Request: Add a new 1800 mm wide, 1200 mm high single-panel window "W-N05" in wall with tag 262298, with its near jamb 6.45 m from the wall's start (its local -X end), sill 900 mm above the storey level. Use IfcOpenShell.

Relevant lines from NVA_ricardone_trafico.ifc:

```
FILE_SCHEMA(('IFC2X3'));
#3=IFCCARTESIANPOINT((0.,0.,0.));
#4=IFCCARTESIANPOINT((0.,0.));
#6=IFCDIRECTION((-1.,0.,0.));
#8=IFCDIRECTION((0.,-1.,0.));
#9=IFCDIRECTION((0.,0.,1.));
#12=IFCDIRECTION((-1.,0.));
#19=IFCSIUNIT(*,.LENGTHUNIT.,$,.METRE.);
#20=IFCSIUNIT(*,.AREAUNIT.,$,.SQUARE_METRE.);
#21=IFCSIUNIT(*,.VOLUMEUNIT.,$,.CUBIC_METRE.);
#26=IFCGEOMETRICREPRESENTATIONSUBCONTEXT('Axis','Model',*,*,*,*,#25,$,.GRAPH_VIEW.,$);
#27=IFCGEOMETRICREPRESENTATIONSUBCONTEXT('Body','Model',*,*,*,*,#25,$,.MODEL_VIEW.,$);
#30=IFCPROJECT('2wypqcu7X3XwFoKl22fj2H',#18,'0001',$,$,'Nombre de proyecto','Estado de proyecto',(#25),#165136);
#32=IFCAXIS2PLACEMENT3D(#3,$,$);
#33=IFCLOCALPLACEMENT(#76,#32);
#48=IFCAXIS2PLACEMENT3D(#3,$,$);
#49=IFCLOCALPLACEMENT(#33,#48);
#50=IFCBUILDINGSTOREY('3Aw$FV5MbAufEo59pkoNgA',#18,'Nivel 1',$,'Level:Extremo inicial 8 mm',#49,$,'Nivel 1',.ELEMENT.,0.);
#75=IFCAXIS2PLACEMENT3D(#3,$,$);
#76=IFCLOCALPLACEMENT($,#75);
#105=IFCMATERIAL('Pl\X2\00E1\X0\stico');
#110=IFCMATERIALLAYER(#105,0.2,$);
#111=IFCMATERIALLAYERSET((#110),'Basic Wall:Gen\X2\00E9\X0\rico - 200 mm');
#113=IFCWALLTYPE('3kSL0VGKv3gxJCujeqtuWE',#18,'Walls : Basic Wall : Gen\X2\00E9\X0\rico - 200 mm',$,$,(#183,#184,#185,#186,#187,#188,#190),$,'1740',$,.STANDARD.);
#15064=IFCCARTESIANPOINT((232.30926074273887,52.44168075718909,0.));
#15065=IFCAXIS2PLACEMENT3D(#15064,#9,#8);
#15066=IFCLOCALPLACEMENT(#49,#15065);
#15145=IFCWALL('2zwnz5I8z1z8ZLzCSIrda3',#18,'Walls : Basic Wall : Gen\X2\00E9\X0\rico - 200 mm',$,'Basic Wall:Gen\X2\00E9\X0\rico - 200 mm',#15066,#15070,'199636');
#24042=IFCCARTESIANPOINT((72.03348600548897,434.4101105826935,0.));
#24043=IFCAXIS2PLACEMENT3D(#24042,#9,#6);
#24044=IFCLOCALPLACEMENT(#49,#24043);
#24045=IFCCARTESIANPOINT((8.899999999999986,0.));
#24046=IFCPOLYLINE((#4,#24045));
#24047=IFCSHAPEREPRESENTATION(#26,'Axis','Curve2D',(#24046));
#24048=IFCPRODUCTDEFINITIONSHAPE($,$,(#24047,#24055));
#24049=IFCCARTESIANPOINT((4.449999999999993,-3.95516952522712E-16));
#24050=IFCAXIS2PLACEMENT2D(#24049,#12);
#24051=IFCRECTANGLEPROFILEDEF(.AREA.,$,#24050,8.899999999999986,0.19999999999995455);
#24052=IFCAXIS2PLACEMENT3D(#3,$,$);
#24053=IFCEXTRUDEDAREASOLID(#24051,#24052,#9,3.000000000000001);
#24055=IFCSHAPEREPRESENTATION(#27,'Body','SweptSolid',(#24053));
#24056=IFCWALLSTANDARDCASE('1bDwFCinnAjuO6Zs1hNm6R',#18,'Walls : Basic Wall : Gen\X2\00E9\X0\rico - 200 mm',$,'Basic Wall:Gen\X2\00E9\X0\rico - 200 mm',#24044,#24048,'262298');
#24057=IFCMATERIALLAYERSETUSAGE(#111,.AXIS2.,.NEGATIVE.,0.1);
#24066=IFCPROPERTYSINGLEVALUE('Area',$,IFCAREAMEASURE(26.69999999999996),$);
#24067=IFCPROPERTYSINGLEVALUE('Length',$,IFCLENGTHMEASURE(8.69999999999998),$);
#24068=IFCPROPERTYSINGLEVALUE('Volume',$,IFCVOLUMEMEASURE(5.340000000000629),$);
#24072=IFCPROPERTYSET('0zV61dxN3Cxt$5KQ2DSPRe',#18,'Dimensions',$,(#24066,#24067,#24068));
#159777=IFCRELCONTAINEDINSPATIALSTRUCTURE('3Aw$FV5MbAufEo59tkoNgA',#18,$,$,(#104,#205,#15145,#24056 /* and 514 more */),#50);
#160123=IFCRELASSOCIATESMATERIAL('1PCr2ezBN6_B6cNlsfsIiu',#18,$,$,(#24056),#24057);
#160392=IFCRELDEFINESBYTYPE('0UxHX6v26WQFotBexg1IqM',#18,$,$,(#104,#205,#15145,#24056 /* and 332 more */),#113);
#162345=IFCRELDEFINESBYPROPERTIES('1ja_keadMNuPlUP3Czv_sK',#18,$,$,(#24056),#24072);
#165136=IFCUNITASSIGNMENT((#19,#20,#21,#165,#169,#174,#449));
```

```python
import numpy as np
import ifcopenshell
import ifcopenshell.api.feature
import ifcopenshell.api.geometry
import ifcopenshell.api.pset
import ifcopenshell.api.root
import ifcopenshell.api.spatial
import ifcopenshell.api.type
import ifcopenshell.geom
import ifcopenshell.util.element
import ifcopenshell.util.placement
import ifcopenshell.util.representation
import ifcopenshell.util.shape
import ifcopenshell.util.unit

model = ifcopenshell.open("NVA_ricardone_trafico.ifc")
unit_scale = ifcopenshell.util.unit.calculate_unit_scale(model)
area_scale = ifcopenshell.util.unit.calculate_unit_scale(model, "AREAUNIT")
volume_scale = ifcopenshell.util.unit.calculate_unit_scale(model, "VOLUMEUNIT")
settings = ifcopenshell.geom.settings()


def volume(element):
    """Net volume in cubic metres, openings subtracted."""
    shape = ifcopenshell.geom.create_shape(settings, element)
    return ifcopenshell.util.shape.get_volume(shape.geometry)


wall = model.by_guid("1bDwFCinnAjuO6Zs1hNm6R")
storey = ifcopenshell.util.element.get_container(wall, ifc_class="IfcBuildingStorey")
context = ifcopenshell.util.representation.get_context(model, "Model", "Body", "MODEL_VIEW")
before = volume(wall)

width, height, from_end, sill = 1.8, 1.2, 6.45, 0.9  # metres

# The wall runs along its own X axis, and the end named is its -X end.
wall_shape = ifcopenshell.geom.create_shape(settings, wall)
x, y, z = ifcopenshell.util.shape.get_vertices(wall_shape.geometry).T
start = x.min() + from_end
face, thickness = float(y.min()), float(y.max() - y.min())
wall_matrix = ifcopenshell.util.placement.get_local_placement(wall.ObjectPlacement)
level = ifcopenshell.util.placement.get_local_placement(storey.ObjectPlacement)[2, 3]


def in_wall(x, y):
    """Placement at x, y metres in the wall's axes, at sill height."""
    matrix = wall_matrix.copy()
    matrix[:, 3] = wall_matrix @ np.array([x / unit_scale, y / unit_scale, 0.0, 1.0])
    matrix[2, 3] = level + sill / unit_scale
    return matrix


# Opening: a box that overshoots both wall faces by 50 mm.
opening = ifcopenshell.api.root.create_entity(model, ifc_class="IfcOpeningElement")
box = ifcopenshell.api.geometry.add_wall_representation(
    model, context=context, length=width, height=height, thickness=thickness + 0.1
)
ifcopenshell.api.geometry.assign_representation(model, product=opening, representation=box)
ifcopenshell.api.geometry.edit_object_placement(model, product=opening, matrix=in_wall(start, face - 0.05), is_si=False)
ifcopenshell.api.feature.add_feature(model, feature=opening, element=wall)

window = ifcopenshell.api.root.create_entity(model, ifc_class="IfcWindow", name="W-N05")
window.OverallWidth, window.OverallHeight = width / unit_scale, height / unit_scale
body = ifcopenshell.api.geometry.add_window_representation(
    model,
    context=context,
    overall_width=window.OverallWidth,
    overall_height=window.OverallHeight,
    partition_type="SINGLE_PANEL",
)
ifcopenshell.api.geometry.assign_representation(model, product=window, representation=body)
ifcopenshell.api.spatial.assign_container(model, products=[window], relating_structure=storey)
fills = ifcopenshell.api.feature.add_filling(model, opening=opening, element=window)
fills.OwnerHistory = window.OwnerHistory  # required in IFC2X3

# IFC2X3 keeps the operation on the window style.
style = ifcopenshell.api.root.create_entity(model, ifc_class="IfcWindowStyle", name="W-N05")
style.OperationType, style.ConstructionType = "SINGLE_PANEL", "NOTDEFINED"
style.ParameterTakesPrecedence = style.Sizeable = False
ifcopenshell.api.type.assign_type(model, related_objects=[window], relating_type=style)

# Centre the window in the wall's thickness.
ifcopenshell.api.geometry.edit_object_placement(model, product=window, matrix=in_wall(start, face), is_si=False)
window_shape = ifcopenshell.geom.create_shape(settings, window)
depth = ifcopenshell.util.shape.get_vertices(window_shape.geometry)[:, 1]
offset = face + thickness / 2 - (depth.min() + depth.max()) / 2
ifcopenshell.api.geometry.edit_object_placement(model, product=window, matrix=in_wall(start, offset), is_si=False)

after = volume(wall)

# Update the wall's stored quantities.
pset = model.by_id(ifcopenshell.util.element.get_pset(wall, "Dimensions", should_inherit=False)["id"])
ifcopenshell.api.pset.edit_pset(model, pset=pset, properties={
    "Area": model.create_entity("IfcAreaMeasure", after / thickness / area_scale),
    "Volume": model.create_entity("IfcVolumeMeasure", after / volume_scale),
})

print(f"wall volume {before:.3f} -> {after:.3f} m3")

model.write("NVA_ricardone_trafico_edited.ifc")
```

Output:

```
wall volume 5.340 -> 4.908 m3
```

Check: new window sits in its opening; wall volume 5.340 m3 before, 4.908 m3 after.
